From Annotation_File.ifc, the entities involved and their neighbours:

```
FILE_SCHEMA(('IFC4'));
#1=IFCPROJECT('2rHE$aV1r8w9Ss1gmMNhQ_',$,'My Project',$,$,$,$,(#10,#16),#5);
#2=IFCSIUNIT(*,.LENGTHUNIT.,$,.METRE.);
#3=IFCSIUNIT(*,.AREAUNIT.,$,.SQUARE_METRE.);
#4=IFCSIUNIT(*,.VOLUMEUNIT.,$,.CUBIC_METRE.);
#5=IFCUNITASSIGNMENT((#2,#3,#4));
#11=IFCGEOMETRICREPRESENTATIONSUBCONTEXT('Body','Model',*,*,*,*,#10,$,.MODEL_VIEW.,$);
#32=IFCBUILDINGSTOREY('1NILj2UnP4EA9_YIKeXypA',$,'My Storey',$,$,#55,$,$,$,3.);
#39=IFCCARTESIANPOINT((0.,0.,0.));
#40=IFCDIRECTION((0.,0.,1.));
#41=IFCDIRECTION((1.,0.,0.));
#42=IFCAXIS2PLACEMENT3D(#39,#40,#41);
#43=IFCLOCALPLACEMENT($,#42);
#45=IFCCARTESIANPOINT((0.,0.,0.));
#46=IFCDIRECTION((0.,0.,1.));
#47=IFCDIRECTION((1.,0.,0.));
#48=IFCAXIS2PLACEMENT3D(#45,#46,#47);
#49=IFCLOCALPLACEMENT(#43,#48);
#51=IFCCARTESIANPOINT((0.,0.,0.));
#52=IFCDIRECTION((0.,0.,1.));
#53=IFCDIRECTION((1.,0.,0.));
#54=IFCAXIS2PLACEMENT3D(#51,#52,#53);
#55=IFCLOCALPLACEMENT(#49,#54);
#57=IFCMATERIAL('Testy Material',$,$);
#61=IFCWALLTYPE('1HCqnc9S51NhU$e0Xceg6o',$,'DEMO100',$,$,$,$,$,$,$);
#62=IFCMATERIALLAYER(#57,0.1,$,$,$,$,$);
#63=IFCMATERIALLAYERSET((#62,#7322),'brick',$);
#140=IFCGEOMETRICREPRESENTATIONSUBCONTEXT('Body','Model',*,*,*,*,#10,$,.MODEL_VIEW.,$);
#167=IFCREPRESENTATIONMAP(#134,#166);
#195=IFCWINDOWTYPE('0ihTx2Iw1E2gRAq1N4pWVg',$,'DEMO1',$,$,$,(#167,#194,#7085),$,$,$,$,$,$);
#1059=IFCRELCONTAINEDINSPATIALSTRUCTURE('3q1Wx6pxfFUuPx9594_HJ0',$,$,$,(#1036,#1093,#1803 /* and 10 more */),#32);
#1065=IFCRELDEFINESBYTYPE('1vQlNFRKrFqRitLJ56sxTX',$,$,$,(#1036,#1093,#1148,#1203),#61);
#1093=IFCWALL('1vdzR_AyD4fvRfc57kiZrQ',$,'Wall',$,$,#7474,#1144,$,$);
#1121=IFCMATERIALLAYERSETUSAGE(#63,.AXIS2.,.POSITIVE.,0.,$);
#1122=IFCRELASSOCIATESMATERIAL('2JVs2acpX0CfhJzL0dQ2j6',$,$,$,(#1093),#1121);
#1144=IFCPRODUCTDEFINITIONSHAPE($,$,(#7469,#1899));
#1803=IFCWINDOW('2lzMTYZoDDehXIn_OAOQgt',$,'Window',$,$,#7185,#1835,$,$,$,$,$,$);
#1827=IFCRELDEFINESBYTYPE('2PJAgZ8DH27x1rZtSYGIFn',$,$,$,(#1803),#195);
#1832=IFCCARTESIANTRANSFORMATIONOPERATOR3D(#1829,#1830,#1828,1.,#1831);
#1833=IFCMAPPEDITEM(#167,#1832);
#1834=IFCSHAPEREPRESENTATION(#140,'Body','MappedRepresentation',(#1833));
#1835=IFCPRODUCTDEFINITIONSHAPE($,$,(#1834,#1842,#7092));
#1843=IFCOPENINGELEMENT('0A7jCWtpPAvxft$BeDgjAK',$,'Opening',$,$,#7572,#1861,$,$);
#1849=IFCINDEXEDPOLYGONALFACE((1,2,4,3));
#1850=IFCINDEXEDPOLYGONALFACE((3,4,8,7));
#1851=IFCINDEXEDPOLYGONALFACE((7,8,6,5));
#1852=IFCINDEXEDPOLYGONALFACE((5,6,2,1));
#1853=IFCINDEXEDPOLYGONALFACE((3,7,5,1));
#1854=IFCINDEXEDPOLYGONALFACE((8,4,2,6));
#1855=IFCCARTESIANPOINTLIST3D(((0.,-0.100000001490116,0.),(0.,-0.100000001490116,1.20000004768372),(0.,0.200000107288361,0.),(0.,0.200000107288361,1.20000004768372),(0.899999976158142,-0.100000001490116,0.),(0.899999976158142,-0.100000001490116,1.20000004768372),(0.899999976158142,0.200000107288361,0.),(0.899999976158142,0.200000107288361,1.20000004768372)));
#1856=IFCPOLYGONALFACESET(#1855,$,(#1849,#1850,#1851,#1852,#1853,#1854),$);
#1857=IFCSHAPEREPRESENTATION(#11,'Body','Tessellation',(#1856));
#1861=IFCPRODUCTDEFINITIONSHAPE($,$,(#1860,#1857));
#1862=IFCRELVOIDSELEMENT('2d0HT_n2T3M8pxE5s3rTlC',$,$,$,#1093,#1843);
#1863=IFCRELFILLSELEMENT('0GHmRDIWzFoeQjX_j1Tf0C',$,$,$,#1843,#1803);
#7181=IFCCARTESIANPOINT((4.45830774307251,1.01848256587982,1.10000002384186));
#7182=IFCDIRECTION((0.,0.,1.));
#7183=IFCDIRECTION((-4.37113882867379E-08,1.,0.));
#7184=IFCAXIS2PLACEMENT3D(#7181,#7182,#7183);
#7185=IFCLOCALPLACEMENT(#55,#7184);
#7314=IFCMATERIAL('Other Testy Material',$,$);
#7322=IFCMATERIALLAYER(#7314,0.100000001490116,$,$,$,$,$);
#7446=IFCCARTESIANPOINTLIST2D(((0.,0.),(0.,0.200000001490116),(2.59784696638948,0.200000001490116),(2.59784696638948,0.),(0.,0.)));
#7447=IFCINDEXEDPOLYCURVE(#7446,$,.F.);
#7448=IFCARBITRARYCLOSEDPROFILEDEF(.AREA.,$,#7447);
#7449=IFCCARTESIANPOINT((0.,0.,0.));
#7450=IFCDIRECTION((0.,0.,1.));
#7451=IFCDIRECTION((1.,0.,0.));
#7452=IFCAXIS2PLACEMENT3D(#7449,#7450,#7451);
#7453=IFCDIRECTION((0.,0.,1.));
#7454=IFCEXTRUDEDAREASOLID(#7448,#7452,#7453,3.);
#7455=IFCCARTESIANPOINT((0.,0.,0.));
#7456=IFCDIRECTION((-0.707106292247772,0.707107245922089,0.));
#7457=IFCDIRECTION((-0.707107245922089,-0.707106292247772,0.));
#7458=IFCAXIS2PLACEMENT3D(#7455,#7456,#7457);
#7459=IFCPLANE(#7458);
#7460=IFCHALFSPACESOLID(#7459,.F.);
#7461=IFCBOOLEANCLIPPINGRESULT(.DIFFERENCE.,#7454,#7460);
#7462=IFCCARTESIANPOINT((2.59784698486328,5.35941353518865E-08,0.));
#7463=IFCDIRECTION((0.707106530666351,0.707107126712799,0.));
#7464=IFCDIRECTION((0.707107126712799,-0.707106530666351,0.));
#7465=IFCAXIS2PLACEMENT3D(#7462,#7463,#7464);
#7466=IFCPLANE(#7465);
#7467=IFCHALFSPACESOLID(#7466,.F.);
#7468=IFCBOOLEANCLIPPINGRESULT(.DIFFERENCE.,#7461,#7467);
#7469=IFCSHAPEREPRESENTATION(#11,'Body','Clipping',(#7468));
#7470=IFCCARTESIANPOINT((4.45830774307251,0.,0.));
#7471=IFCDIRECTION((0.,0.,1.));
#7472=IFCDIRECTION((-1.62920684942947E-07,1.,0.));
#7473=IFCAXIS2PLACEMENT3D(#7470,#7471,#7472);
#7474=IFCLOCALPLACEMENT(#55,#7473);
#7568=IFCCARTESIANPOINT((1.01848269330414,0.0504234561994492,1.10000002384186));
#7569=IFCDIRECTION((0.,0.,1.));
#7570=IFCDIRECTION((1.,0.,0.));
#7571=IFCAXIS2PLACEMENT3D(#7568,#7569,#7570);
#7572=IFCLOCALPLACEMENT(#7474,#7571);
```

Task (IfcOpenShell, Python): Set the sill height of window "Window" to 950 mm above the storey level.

```python
import numpy as np
import ifcopenshell
import ifcopenshell.api.geometry
import ifcopenshell.geom
import ifcopenshell.util.element
import ifcopenshell.util.placement
import ifcopenshell.util.shape
import ifcopenshell.util.unit

model = ifcopenshell.open("Annotation_File.ifc")
unit_scale = ifcopenshell.util.unit.calculate_unit_scale(model)

window = model.by_id(1803)
opening = window.FillsVoids[0].RelatingOpeningElement
storey = ifcopenshell.util.element.get_container(window, ifc_class="IfcBuildingStorey")
level = ifcopenshell.util.placement.get_local_placement(storey.ObjectPlacement)[2, 3]

# The opening's origin need not be at the sill, so measure its lowest point.
shape = ifcopenshell.geom.create_shape(ifcopenshell.geom.settings(), opening)
bottom = ifcopenshell.util.shape.get_shape_bottom_elevation(shape, shape.geometry) / unit_scale
dz = level + 0.95 / unit_scale - bottom

shift = np.array([0.0, 0.0, dz])
# The window is not placed relative to its opening, so move both.
for product in (opening, window):
    matrix = ifcopenshell.util.placement.get_local_placement(product.ObjectPlacement)
    matrix[:3, 3] += shift
    ifcopenshell.api.geometry.edit_object_placement(model, product=product, matrix=matrix, is_si=False)

print(f"moved by {dz * unit_scale:+.3f} m")

model.write("Annotation_File_edited.ifc")
```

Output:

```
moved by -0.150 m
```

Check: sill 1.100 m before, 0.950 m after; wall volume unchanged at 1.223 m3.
